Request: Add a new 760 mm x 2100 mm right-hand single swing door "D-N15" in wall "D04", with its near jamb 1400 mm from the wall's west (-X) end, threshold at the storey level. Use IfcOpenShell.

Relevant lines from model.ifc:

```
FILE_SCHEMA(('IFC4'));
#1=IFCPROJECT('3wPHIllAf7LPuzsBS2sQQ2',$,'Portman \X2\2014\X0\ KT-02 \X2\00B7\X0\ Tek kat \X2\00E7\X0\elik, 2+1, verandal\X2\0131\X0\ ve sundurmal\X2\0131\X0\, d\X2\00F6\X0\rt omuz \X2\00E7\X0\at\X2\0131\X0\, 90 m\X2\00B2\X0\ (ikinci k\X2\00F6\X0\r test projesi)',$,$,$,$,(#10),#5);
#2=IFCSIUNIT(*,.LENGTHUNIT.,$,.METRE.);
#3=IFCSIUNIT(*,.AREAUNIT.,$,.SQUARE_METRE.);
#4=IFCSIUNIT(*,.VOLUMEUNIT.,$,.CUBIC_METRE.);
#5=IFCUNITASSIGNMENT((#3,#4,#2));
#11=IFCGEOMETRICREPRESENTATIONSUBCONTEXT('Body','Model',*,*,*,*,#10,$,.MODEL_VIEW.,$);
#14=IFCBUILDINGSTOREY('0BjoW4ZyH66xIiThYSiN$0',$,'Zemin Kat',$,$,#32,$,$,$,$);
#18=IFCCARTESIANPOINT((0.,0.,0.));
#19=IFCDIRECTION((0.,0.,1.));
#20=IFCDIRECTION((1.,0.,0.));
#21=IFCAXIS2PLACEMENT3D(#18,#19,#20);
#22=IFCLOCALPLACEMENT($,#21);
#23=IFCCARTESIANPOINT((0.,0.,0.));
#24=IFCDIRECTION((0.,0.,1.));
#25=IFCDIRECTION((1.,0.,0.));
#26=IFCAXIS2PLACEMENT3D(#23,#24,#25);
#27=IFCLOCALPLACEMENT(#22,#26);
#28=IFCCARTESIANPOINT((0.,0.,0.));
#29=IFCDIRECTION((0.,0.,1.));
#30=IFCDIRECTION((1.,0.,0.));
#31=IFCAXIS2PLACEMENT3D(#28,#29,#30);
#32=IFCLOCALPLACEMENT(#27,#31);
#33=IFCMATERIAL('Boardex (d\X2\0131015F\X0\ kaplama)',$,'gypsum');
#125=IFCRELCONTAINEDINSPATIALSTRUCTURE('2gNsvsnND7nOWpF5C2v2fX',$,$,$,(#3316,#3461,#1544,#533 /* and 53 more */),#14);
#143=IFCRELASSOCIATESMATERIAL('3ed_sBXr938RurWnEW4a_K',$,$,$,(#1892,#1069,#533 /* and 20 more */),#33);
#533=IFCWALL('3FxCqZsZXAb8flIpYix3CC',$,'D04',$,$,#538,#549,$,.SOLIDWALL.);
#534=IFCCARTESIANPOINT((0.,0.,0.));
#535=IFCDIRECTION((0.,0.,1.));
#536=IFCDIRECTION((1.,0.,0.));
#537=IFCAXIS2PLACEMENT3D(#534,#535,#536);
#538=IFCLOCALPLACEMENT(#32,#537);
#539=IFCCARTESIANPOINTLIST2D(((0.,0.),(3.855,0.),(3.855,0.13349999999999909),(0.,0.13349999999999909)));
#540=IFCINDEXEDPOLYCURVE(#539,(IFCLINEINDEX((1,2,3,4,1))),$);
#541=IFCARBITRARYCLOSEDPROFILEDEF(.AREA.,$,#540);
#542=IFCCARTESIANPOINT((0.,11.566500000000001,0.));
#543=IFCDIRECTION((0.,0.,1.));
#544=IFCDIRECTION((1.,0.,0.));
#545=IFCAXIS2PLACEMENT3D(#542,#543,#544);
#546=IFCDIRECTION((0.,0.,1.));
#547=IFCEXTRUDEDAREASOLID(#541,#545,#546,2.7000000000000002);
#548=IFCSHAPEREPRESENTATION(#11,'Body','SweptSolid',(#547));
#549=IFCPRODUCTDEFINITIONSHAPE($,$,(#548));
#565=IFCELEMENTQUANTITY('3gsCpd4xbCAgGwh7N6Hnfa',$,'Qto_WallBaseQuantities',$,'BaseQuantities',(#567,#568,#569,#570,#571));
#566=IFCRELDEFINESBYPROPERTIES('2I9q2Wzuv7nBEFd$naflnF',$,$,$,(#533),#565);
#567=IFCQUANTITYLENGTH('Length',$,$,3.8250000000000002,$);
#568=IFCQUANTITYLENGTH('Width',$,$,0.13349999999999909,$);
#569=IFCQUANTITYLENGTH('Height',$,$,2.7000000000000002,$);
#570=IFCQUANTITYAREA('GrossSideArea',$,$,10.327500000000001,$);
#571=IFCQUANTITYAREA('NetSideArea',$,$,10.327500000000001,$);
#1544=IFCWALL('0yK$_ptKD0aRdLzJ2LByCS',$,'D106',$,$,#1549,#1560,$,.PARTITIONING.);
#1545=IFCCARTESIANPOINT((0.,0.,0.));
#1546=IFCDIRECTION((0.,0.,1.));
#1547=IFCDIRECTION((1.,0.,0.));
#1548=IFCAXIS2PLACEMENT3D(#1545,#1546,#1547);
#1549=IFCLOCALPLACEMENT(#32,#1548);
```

```python
import numpy as np
import ifcopenshell
import ifcopenshell.api.feature
import ifcopenshell.api.geometry
import ifcopenshell.api.pset
import ifcopenshell.api.root
import ifcopenshell.api.spatial
import ifcopenshell.geom
import ifcopenshell.util.element
import ifcopenshell.util.placement
import ifcopenshell.util.representation
import ifcopenshell.util.shape
import ifcopenshell.util.unit

model = ifcopenshell.open("model.ifc")
unit_scale = ifcopenshell.util.unit.calculate_unit_scale(model)
area_scale = ifcopenshell.util.unit.calculate_unit_scale(model, "AREAUNIT")
settings = ifcopenshell.geom.settings()


def volume(element):
    """Net volume in cubic metres, openings subtracted."""
    shape = ifcopenshell.geom.create_shape(settings, element)
    return ifcopenshell.util.shape.get_volume(shape.geometry)


wall = model.by_id(533)
storey = ifcopenshell.util.element.get_container(wall, ifc_class="IfcBuildingStorey")
context = ifcopenshell.util.representation.get_context(model, "Model", "Body", "MODEL_VIEW")
before = volume(wall)

width, height, from_end, sill = 0.76, 2.1, 1.4, 0.0  # metres

# The wall runs along its own X axis, and the end named is its -X end.
wall_shape = ifcopenshell.geom.create_shape(settings, wall)
x, y, z = ifcopenshell.util.shape.get_vertices(wall_shape.geometry).T
start = x.min() + from_end
face, thickness = float(y.min()), float(y.max() - y.min())
wall_matrix = ifcopenshell.util.placement.get_local_placement(wall.ObjectPlacement)
level = ifcopenshell.util.placement.get_local_placement(storey.ObjectPlacement)[2, 3]


def in_wall(x, y):
    """Placement at x, y metres in the wall's axes, at sill height."""
    matrix = wall_matrix.copy()
    matrix[:, 3] = wall_matrix @ np.array([x / unit_scale, y / unit_scale, 0.0, 1.0])
    matrix[2, 3] = level + sill / unit_scale
    return matrix


# Opening: a box that overshoots both wall faces by 50 mm.
opening = ifcopenshell.api.root.create_entity(model, ifc_class="IfcOpeningElement", predefined_type="OPENING")
box = ifcopenshell.api.geometry.add_wall_representation(
    model, context=context, length=width, height=height, thickness=thickness + 0.1
)
ifcopenshell.api.geometry.assign_representation(model, product=opening, representation=box)
ifcopenshell.api.geometry.edit_object_placement(model, product=opening, matrix=in_wall(start, face - 0.05), is_si=False)
ifcopenshell.api.feature.add_feature(model, feature=opening, element=wall)

door = ifcopenshell.api.root.create_entity(model, ifc_class="IfcDoor", name="D-N15", predefined_type="DOOR")
door.OverallWidth, door.OverallHeight = width / unit_scale, height / unit_scale
door.OperationType = "SINGLE_SWING_RIGHT"
body = ifcopenshell.api.geometry.add_door_representation(
    model,
    context=context,
    overall_width=door.OverallWidth,
    overall_height=door.OverallHeight,
    operation_type="SINGLE_SWING_RIGHT",
    lining_properties={"LiningDepth": thickness / unit_scale, "ThresholdDepth": thickness / unit_scale},
)
ifcopenshell.api.geometry.assign_representation(model, product=door, representation=body)
ifcopenshell.api.spatial.assign_container(model, products=[door], relating_structure=storey)
ifcopenshell.api.feature.add_filling(model, opening=opening, element=door)

# The lining spans the wall, so the door starts at the wall face.
ifcopenshell.api.geometry.edit_object_placement(model, product=door, matrix=in_wall(start, face), is_si=False)

after = volume(wall)

# Update the wall's stored quantities.
qto = model.by_id(ifcopenshell.util.element.get_pset(wall, "Qto_WallBaseQuantities", should_inherit=False)["id"])
ifcopenshell.api.pset.edit_qto(model, qto=qto, properties={"NetSideArea": after / thickness / area_scale})

print(f"wall volume {before:.3f} -> {after:.3f} m3")

model.write("model_updated.ifc")
```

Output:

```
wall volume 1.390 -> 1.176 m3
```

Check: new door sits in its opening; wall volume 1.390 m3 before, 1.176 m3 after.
